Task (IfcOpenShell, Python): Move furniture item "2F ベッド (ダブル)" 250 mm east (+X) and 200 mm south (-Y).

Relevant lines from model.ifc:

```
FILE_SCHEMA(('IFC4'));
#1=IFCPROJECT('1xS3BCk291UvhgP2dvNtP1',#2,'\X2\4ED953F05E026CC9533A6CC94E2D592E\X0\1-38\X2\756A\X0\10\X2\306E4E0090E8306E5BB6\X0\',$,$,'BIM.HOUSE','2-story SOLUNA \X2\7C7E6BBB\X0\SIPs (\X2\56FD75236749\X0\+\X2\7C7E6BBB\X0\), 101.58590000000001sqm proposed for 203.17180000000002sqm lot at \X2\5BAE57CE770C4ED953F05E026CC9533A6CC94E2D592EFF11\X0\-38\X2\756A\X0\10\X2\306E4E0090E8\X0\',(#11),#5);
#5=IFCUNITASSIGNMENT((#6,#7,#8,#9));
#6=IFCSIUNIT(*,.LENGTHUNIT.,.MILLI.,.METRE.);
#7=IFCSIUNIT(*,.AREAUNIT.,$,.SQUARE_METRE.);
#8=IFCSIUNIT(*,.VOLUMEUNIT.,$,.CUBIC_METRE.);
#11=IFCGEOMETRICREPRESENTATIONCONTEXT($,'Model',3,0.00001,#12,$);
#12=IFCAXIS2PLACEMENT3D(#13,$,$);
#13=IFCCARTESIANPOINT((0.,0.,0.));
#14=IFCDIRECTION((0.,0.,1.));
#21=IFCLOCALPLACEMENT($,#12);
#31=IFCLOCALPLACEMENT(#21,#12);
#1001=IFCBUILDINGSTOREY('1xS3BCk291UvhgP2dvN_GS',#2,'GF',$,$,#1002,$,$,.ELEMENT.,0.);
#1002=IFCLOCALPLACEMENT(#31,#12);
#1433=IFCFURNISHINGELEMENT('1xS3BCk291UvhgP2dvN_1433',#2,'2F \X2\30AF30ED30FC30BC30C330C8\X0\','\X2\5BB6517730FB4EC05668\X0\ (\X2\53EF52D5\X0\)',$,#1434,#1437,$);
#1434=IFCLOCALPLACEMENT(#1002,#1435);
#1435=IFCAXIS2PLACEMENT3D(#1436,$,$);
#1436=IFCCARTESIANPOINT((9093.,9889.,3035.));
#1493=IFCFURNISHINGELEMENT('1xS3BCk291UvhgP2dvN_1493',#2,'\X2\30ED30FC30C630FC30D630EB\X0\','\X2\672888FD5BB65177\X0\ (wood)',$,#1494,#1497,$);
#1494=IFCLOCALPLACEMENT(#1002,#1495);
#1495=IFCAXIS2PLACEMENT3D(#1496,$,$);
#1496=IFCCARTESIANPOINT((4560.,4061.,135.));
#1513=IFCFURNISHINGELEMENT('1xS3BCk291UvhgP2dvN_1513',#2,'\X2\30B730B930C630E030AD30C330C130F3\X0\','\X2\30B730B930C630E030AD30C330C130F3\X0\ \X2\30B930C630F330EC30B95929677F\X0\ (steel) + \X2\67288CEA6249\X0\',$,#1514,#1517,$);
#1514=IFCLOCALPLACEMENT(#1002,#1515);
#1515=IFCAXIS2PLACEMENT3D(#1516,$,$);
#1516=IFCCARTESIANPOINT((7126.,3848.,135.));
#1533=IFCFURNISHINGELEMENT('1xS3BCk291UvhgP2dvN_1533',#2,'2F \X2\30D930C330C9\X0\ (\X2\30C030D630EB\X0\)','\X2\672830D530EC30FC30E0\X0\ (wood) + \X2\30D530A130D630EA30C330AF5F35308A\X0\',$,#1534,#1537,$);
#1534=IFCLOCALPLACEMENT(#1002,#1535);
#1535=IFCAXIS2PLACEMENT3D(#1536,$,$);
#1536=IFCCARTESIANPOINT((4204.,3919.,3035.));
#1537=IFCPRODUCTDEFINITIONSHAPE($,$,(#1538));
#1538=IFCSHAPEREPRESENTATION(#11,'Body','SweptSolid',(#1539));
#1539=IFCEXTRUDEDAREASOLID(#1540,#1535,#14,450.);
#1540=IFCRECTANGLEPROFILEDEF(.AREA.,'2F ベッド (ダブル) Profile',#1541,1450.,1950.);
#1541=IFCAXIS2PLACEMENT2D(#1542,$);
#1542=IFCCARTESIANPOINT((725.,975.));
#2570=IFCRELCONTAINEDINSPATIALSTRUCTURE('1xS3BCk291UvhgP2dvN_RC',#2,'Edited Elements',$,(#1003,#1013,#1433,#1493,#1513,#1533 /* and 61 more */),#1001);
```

```python
import ifcopenshell
import ifcopenshell.api.geometry
import ifcopenshell.util.placement
import ifcopenshell.util.unit

model = ifcopenshell.open("model.ifc")
unit_scale = ifcopenshell.util.unit.calculate_unit_scale(model)

item = model.by_guid("1xS3BCk291UvhgP2dvN_1533")
matrix = ifcopenshell.util.placement.get_local_placement(item.ObjectPlacement)
matrix[0, 3] += 0.25 / unit_scale
matrix[1, 3] -= 0.2 / unit_scale
ifcopenshell.api.geometry.edit_object_placement(model, product=item, matrix=matrix, is_si=False)

print(ifcopenshell.util.placement.get_local_placement(item.ObjectPlacement).round(3) + 0.0)

model.write("model_edited.ifc")
```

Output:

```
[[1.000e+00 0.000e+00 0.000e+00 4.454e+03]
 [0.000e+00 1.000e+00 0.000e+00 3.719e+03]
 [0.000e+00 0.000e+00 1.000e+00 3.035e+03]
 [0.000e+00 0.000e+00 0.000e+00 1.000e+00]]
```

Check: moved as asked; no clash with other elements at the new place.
